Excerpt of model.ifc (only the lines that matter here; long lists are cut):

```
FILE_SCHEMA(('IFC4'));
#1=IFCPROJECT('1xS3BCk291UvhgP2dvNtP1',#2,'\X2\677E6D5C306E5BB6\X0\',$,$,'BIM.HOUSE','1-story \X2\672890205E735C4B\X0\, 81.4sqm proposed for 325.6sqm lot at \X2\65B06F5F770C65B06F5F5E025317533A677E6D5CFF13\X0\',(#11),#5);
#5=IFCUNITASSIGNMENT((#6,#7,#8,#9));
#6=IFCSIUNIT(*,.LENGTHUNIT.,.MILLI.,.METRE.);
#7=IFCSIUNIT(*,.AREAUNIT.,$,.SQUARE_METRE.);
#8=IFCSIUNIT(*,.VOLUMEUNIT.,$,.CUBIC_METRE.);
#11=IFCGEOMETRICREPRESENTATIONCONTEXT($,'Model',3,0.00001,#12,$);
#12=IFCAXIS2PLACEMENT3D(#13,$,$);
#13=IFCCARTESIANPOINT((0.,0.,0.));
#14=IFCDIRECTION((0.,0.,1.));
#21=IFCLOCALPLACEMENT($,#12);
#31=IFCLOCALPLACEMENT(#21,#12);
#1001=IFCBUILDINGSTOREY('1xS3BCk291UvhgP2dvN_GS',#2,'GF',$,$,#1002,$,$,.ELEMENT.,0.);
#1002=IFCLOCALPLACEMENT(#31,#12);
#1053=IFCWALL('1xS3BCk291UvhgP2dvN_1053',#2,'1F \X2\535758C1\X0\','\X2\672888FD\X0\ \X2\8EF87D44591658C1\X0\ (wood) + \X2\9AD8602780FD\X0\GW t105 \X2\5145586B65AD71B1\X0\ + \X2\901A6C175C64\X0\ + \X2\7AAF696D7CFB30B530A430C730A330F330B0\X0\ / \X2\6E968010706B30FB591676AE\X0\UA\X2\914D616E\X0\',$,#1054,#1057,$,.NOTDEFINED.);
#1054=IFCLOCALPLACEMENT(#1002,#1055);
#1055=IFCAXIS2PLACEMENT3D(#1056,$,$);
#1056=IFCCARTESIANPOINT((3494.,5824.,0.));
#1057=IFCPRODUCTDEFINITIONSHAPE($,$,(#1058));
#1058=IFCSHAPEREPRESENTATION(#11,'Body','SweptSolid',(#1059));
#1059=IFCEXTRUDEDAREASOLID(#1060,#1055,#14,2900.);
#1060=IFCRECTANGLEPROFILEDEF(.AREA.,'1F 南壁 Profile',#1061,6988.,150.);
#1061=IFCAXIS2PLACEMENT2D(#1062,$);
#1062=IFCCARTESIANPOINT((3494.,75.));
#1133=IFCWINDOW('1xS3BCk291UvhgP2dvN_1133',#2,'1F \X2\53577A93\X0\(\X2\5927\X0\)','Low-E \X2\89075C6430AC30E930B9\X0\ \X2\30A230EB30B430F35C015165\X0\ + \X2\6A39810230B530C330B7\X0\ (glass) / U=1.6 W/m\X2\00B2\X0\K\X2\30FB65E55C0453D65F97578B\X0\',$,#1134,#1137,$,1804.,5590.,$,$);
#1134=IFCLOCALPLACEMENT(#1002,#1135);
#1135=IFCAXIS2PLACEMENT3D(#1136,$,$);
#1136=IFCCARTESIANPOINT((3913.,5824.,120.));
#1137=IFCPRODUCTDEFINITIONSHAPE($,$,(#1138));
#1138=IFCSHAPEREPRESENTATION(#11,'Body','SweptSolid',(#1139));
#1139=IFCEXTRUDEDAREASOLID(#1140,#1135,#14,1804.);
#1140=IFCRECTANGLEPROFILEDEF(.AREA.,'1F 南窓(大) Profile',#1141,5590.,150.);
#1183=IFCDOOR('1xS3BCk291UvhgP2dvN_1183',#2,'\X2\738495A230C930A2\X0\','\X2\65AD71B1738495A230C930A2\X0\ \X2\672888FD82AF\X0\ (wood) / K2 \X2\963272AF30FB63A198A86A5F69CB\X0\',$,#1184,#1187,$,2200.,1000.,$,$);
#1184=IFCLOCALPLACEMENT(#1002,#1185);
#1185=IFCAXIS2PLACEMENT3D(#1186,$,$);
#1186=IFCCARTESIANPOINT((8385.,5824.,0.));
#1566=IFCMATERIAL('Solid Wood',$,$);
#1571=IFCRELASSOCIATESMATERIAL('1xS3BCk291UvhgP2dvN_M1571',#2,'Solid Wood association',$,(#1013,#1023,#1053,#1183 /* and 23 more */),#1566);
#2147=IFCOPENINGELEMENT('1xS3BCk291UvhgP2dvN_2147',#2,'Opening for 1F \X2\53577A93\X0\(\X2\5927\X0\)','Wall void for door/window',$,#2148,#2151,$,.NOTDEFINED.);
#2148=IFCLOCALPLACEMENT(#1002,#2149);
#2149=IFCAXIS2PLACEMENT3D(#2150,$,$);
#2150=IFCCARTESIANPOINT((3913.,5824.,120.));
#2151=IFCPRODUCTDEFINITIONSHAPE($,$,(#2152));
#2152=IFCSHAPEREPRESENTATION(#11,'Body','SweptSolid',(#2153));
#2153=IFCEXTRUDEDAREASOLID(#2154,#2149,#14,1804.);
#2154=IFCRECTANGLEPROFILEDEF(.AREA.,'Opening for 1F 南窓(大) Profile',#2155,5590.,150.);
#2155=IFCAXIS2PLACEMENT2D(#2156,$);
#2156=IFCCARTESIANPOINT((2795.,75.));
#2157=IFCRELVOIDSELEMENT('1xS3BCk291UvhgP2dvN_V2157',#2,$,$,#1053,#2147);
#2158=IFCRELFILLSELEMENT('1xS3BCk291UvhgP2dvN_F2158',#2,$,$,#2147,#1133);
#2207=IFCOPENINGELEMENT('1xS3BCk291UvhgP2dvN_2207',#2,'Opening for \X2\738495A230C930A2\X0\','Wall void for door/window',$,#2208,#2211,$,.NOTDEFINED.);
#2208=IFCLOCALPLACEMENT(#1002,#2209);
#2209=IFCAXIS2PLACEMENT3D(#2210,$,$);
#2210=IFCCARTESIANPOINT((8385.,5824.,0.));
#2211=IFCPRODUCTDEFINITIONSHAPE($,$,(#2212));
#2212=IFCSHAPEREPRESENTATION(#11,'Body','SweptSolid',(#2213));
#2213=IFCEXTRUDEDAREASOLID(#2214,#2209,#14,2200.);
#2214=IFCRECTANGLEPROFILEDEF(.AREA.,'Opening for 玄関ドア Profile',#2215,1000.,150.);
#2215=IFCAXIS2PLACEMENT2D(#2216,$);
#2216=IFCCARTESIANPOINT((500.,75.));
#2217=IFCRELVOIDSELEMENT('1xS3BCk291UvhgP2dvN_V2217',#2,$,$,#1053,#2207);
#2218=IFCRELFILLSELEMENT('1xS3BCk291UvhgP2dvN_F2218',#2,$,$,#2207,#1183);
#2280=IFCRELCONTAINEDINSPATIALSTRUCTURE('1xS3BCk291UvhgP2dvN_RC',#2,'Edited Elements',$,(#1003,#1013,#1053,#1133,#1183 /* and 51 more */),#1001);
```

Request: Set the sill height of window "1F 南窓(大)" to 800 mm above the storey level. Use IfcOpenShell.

```python
import numpy as np
import ifcopenshell
import ifcopenshell.api.geometry
import ifcopenshell.geom
import ifcopenshell.util.element
import ifcopenshell.util.placement
import ifcopenshell.util.shape
import ifcopenshell.util.unit

model = ifcopenshell.open("model.ifc")
unit_scale = ifcopenshell.util.unit.calculate_unit_scale(model)

window = model.by_id(1133)
opening = window.FillsVoids[0].RelatingOpeningElement
storey = ifcopenshell.util.element.get_container(window, ifc_class="IfcBuildingStorey")
level = ifcopenshell.util.placement.get_local_placement(storey.ObjectPlacement)[2, 3]

# The opening's origin need not be at the sill, so measure its lowest point.
shape = ifcopenshell.geom.create_shape(ifcopenshell.geom.settings(), opening)
bottom = ifcopenshell.util.shape.get_shape_bottom_elevation(shape, shape.geometry) / unit_scale
dz = level + 0.8 / unit_scale - bottom

shift = np.array([0.0, 0.0, dz])
# The window is not placed relative to its opening, so move both.
for product in (opening, window):
    matrix = ifcopenshell.util.placement.get_local_placement(product.ObjectPlacement)
    matrix[:3, 3] += shift
    ifcopenshell.api.geometry.edit_object_placement(model, product=product, matrix=matrix, is_si=False)

print(f"moved by {dz * unit_scale:+.3f} m")

model.write("model_updated.ifc")
```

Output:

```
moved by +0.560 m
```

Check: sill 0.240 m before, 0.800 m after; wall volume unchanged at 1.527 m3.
